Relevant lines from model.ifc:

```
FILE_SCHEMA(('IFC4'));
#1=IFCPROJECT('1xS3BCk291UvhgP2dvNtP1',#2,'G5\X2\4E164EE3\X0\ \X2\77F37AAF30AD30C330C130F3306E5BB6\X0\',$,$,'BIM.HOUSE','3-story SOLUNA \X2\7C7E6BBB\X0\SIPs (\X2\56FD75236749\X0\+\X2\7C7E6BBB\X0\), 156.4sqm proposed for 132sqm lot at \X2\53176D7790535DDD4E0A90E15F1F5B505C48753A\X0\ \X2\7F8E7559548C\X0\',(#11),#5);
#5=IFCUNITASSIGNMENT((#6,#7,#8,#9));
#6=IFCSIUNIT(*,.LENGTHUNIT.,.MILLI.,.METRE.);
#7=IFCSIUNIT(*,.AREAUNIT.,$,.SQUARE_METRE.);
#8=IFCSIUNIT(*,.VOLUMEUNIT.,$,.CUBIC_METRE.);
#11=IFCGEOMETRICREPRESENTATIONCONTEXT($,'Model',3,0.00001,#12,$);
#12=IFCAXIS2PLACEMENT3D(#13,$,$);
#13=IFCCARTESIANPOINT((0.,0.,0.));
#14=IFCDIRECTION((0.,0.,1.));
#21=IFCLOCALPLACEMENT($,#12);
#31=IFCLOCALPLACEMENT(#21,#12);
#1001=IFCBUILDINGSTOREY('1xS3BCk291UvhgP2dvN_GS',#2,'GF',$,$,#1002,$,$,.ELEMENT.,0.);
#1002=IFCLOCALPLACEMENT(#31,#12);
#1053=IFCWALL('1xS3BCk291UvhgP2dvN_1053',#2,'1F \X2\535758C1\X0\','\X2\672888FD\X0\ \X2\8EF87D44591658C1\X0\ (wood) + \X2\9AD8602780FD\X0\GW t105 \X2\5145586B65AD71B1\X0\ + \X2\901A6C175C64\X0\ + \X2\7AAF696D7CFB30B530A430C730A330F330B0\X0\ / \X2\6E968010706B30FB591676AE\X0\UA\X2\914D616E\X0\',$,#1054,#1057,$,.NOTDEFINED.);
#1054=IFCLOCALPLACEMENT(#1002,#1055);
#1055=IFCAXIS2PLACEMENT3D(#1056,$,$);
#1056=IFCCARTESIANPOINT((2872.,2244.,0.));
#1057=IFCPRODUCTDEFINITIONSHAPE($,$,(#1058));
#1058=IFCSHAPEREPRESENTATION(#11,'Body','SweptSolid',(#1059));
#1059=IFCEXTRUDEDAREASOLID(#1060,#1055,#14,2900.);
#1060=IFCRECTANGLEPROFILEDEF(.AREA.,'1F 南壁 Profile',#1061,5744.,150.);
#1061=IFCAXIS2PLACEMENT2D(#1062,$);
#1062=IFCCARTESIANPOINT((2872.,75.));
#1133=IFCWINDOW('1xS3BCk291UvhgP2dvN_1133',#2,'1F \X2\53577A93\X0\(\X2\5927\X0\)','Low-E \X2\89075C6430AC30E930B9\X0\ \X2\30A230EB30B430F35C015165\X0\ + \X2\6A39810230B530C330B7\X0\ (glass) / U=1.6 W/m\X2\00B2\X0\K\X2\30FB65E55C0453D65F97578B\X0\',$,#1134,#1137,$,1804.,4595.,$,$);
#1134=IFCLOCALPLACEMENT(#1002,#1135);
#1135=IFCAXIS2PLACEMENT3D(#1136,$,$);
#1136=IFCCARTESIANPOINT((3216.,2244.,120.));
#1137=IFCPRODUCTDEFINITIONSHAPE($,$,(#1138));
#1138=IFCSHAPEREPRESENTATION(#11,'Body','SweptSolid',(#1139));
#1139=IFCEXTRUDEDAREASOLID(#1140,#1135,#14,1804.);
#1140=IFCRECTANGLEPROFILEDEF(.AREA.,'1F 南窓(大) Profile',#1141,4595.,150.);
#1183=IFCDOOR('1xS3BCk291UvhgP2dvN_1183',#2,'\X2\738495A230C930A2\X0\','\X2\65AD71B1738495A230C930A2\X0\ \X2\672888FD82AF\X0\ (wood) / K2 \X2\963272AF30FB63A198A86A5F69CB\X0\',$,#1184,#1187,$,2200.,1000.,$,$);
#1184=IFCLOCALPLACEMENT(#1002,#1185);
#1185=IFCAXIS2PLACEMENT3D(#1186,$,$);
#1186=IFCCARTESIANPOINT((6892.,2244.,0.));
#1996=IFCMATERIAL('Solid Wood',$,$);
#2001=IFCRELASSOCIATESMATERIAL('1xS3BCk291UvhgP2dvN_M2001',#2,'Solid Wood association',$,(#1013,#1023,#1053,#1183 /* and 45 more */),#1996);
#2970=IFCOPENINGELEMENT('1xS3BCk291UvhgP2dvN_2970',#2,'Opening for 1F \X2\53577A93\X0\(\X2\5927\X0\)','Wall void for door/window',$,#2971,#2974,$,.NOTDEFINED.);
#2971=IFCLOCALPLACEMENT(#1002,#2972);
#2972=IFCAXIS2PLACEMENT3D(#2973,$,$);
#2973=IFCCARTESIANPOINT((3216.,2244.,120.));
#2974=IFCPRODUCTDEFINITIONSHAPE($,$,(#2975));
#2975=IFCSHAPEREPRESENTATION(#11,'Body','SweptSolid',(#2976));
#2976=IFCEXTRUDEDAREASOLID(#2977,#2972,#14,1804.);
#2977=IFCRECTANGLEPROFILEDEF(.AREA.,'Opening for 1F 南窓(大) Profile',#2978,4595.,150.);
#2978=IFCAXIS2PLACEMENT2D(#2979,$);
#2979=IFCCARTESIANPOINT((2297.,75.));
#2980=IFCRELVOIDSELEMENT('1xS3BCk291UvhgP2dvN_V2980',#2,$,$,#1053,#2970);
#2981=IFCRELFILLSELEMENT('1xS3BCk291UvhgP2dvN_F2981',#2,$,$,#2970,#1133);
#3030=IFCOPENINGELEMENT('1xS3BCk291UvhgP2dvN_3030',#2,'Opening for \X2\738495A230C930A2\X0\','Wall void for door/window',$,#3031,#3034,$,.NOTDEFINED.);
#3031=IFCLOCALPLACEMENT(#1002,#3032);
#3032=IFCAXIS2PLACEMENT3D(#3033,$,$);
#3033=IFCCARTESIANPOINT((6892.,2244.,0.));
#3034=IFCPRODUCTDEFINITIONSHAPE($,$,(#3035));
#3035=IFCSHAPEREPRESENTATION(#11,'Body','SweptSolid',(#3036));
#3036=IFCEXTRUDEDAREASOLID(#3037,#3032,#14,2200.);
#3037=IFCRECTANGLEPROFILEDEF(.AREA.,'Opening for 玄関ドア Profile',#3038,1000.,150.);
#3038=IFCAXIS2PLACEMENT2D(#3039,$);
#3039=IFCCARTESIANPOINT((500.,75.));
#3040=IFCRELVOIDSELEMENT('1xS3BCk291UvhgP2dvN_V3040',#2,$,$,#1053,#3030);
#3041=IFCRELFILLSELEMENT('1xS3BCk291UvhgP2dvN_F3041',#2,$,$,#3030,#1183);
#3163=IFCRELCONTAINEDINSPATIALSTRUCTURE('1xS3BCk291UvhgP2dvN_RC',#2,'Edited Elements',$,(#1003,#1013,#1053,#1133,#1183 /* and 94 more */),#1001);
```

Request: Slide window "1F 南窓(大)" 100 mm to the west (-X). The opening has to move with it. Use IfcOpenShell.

```python
import ifcopenshell
import ifcopenshell.api.geometry
import ifcopenshell.util.placement

model = ifcopenshell.open("model.ifc")

window = model.by_guid("1xS3BCk291UvhgP2dvN_1133")
opening = window.FillsVoids[0].RelatingOpeningElement
wall = opening.VoidsElements[0].RelatingBuildingElement

wall_matrix = ifcopenshell.util.placement.get_local_placement(wall.ObjectPlacement)
shift = wall_matrix[:3, 0] * -100.0
before = ifcopenshell.util.placement.get_local_placement(window.ObjectPlacement)[:3, 3].copy()

# The window is not placed relative to its opening, so move both.
for product in (opening, window):
    matrix = ifcopenshell.util.placement.get_local_placement(product.ObjectPlacement)
    matrix[:3, 3] += shift
    ifcopenshell.api.geometry.edit_object_placement(model, product=product, matrix=matrix, is_si=False)

after = ifcopenshell.util.placement.get_local_placement(window.ObjectPlacement)[:3, 3]
print("window moved by", (after - before).round(3) + 0.0)

model.write("model_edited.ifc")
```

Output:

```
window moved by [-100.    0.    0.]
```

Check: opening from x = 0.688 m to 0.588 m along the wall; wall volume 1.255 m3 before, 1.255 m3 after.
